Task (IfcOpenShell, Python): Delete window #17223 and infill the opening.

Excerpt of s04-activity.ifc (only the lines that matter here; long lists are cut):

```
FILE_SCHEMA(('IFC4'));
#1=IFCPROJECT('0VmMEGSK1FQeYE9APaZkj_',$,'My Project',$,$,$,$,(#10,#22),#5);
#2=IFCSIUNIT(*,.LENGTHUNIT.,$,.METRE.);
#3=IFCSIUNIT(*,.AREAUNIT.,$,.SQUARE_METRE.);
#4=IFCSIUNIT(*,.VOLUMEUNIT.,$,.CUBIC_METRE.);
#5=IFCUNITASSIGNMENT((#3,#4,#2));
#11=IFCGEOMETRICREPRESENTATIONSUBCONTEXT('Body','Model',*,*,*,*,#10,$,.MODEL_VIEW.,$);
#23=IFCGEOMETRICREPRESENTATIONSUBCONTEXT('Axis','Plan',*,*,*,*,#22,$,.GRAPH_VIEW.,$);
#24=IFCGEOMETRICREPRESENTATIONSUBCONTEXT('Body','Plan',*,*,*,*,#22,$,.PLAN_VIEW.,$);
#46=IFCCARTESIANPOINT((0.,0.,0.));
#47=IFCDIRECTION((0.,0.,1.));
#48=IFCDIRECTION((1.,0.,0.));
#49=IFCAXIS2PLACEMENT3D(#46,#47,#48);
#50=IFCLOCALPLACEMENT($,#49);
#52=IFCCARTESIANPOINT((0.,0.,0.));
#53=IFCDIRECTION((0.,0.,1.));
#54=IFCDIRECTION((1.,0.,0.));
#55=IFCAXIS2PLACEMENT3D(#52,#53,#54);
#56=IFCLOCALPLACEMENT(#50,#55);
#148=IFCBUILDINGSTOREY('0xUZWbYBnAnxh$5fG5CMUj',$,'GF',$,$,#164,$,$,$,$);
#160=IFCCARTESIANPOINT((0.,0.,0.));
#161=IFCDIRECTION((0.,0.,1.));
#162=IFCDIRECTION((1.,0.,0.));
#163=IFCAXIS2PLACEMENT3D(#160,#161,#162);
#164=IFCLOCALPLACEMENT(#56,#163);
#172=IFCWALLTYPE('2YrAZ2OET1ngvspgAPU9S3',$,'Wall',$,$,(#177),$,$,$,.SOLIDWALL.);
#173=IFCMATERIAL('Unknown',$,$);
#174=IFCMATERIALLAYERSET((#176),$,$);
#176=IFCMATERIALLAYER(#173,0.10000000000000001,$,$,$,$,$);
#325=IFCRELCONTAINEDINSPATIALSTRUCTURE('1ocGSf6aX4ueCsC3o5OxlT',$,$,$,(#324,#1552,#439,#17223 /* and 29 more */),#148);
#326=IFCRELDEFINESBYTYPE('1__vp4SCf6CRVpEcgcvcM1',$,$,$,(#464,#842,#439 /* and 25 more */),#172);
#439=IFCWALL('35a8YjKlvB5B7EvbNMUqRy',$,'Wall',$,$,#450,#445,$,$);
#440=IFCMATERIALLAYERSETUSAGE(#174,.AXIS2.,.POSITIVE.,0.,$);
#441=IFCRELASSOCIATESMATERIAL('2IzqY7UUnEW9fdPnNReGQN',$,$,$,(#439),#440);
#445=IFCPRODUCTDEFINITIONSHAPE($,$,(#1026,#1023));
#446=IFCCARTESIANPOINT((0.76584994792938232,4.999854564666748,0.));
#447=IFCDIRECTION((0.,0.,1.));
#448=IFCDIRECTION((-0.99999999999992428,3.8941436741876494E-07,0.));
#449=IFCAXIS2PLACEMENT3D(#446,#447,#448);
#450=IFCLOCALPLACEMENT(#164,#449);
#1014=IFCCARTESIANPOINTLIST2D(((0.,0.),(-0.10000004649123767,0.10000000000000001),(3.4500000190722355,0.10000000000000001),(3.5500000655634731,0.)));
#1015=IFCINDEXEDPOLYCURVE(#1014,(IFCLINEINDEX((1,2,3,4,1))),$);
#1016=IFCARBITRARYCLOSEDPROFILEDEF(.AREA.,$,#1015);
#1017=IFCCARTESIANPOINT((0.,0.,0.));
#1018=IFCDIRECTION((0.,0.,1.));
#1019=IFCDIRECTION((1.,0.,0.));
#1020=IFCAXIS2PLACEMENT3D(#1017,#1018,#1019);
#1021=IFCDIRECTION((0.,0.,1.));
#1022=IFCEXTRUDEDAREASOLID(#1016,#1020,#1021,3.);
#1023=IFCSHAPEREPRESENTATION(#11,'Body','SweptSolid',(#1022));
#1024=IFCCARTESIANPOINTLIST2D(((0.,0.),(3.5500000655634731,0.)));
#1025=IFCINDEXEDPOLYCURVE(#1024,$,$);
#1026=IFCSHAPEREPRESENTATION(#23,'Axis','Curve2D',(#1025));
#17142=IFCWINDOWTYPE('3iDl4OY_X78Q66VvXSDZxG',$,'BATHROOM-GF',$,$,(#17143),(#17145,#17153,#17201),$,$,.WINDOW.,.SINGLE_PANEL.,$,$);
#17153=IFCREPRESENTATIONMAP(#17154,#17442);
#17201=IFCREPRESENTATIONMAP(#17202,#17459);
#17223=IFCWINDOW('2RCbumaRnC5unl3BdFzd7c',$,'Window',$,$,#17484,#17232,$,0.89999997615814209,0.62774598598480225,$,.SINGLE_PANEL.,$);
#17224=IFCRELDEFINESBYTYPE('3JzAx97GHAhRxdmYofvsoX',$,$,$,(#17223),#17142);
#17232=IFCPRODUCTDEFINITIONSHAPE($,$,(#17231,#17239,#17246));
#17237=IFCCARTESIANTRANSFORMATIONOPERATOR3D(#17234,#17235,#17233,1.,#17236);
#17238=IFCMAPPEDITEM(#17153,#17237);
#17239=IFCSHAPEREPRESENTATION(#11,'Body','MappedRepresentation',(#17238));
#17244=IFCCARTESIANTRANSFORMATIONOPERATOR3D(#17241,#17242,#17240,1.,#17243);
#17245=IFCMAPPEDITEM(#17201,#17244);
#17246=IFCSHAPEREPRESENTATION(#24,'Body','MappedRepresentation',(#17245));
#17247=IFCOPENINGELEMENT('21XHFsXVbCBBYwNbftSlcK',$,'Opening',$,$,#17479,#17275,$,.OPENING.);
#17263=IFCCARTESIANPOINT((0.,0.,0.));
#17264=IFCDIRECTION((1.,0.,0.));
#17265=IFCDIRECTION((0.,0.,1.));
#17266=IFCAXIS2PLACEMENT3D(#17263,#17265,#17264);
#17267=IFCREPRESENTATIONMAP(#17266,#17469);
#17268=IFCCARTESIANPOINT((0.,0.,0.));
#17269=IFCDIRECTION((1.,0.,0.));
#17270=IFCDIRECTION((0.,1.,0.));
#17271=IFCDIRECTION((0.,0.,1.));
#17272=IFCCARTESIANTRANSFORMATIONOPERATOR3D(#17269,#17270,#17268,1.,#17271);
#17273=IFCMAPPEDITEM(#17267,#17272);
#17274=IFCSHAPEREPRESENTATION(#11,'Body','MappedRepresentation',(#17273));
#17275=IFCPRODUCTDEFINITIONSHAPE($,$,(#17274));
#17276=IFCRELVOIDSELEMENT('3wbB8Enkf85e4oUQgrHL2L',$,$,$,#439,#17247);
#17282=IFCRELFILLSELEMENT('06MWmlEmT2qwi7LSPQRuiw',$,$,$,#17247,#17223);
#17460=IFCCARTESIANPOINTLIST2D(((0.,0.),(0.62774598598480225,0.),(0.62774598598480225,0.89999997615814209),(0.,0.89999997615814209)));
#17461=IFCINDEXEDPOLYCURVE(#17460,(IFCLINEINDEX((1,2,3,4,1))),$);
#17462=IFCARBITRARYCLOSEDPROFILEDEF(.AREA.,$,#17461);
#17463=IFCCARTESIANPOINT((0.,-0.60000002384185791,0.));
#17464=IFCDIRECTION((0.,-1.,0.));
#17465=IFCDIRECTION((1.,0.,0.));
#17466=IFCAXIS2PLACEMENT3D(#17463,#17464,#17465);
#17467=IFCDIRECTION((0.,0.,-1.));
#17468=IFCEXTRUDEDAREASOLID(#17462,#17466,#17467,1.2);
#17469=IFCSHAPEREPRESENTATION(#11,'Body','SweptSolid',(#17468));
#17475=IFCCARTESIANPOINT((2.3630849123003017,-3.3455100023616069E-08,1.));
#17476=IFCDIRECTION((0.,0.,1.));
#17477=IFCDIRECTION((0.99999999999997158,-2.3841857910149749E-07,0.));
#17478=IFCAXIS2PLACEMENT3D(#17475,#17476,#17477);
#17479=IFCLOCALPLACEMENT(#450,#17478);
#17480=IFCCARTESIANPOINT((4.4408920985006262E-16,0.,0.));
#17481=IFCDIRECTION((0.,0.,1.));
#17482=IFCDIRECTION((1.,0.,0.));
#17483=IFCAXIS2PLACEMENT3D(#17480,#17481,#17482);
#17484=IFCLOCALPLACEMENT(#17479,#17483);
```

```python
import ifcopenshell
import ifcopenshell.api.feature
import ifcopenshell.api.root
import ifcopenshell.geom
import ifcopenshell.util.shape

model = ifcopenshell.open("s04-activity.ifc")
settings = ifcopenshell.geom.settings()


def volume(element):
    """Net volume in cubic metres, openings subtracted."""
    shape = ifcopenshell.geom.create_shape(settings, element)
    return ifcopenshell.util.shape.get_volume(shape.geometry)


window = model.by_guid("2RCbumaRnC5unl3BdFzd7c")
opening = window.FillsVoids[0].RelatingOpeningElement
wall = opening.VoidsElements[0].RelatingBuildingElement
before = volume(wall)

ifcopenshell.api.root.remove_product(model, product=window)
ifcopenshell.api.feature.remove_feature(model, feature=opening)

after = volume(wall)

print(f"wall volume {before:.3f} -> {after:.3f} m3")

model.write("s04-activity_v2.ifc")
```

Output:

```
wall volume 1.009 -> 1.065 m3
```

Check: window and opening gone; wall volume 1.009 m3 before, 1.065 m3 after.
